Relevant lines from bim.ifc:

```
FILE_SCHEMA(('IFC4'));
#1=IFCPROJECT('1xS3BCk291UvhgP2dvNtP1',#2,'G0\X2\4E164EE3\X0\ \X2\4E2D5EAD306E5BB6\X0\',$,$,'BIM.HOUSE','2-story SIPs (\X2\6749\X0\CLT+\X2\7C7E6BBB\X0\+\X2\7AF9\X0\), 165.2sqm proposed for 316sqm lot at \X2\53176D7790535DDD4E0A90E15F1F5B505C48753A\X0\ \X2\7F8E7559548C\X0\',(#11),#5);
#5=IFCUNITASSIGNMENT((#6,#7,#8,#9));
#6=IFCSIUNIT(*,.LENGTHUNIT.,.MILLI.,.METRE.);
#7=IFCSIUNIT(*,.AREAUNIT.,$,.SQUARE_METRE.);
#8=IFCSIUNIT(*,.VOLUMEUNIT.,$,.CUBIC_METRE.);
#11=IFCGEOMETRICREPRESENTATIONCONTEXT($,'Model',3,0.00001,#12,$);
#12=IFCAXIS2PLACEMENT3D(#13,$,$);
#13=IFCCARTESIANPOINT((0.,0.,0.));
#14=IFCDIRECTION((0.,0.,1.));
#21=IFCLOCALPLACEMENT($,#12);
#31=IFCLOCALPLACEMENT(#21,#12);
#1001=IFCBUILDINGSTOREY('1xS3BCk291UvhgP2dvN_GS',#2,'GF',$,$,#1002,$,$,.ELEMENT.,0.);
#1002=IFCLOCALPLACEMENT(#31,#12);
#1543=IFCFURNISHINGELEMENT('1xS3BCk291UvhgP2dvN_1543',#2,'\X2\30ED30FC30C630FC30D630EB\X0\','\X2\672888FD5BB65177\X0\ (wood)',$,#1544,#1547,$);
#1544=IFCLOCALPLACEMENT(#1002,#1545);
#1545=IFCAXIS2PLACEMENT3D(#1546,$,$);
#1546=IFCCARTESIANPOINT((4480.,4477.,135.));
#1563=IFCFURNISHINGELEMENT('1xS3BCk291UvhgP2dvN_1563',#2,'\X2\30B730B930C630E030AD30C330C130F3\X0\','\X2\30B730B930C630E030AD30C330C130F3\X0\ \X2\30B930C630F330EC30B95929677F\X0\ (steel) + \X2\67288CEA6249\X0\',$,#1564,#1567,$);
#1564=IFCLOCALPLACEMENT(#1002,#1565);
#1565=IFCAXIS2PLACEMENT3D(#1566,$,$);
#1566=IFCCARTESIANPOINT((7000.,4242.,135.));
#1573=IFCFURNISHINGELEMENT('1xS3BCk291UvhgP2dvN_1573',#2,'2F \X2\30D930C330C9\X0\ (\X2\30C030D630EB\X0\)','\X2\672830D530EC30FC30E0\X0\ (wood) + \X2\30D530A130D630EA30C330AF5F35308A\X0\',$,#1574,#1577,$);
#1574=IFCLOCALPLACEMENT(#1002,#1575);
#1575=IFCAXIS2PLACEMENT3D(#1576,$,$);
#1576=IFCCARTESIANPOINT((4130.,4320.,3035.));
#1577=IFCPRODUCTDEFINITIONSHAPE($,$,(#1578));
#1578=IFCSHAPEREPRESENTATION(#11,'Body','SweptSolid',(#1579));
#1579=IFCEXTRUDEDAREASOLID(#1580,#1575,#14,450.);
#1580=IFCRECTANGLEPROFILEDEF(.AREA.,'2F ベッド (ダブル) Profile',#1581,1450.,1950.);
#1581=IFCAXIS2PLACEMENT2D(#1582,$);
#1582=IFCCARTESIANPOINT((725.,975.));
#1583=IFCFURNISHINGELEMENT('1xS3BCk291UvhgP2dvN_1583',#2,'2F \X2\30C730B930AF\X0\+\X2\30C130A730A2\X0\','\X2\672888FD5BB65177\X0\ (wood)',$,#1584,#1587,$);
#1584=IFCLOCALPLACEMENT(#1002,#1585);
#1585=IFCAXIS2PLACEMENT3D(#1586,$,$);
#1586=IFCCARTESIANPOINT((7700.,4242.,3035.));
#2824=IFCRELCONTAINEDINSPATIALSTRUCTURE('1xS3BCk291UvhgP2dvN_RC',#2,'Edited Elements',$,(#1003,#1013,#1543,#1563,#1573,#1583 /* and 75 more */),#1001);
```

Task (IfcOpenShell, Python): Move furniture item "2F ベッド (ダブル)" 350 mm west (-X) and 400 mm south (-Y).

```python
import ifcopenshell
import ifcopenshell.api.geometry
import ifcopenshell.util.placement
import ifcopenshell.util.unit

model = ifcopenshell.open("bim.ifc")
unit_scale = ifcopenshell.util.unit.calculate_unit_scale(model)

item = model.by_guid("1xS3BCk291UvhgP2dvN_1573")
matrix = ifcopenshell.util.placement.get_local_placement(item.ObjectPlacement)
matrix[0, 3] -= 0.35 / unit_scale
matrix[1, 3] -= 0.4 / unit_scale
ifcopenshell.api.geometry.edit_object_placement(model, product=item, matrix=matrix, is_si=False)

print(ifcopenshell.util.placement.get_local_placement(item.ObjectPlacement).round(3) + 0.0)

model.write("bim-out.ifc")
```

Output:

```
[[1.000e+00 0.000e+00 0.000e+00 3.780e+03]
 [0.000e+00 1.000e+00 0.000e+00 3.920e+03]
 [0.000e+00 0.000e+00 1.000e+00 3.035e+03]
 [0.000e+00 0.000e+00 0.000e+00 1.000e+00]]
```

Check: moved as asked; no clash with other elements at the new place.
